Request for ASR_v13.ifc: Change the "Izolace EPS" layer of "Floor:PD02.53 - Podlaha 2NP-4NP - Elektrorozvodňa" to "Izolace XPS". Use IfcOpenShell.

First a look at what the model holds.

```python
import ifcopenshell
import ifcopenshell.util.element

model = ifcopenshell.open("ASR_v13.ifc")
print(model.schema)
for layer_set in model.by_type("IfcMaterialLayerSet"):
    if layer_set.LayerSetName == "Floor:PD02.53 - Podlaha 2NP-4NP - Elektrorozvodňa":
        for layer in layer_set.MaterialLayers:
            print(layer.id(), layer.Material and layer.Material.Name, layer.LayerThickness, sep=" | ")
        print(len(ifcopenshell.util.element.get_elements_by_material(model, layer_set)), "elements and types use it")
print(sorted(m.Name for m in model.by_type("IfcMaterial") if m.Name)[:60])
```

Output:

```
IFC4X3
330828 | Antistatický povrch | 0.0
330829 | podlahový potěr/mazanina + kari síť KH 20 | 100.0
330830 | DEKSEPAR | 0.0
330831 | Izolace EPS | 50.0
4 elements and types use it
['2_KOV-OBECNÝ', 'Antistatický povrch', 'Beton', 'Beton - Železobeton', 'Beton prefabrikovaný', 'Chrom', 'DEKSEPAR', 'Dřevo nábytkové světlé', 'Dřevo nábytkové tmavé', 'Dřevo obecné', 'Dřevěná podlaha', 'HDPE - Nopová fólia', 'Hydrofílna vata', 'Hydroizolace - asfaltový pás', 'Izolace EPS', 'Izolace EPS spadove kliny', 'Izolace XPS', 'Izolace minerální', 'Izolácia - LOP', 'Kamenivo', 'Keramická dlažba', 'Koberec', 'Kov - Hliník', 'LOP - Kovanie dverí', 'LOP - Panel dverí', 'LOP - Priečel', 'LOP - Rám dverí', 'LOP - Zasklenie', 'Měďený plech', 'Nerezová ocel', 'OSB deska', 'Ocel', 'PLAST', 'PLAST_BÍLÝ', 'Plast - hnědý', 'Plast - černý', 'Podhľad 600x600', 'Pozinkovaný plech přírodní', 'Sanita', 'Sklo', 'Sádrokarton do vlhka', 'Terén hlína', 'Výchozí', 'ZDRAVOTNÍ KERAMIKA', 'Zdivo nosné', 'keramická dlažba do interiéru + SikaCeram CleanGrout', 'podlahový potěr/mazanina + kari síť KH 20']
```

```python
import ifcopenshell
import ifcopenshell.api.material

model = ifcopenshell.open("ASR_v13.ifc")

layer_set = next(s for s in model.by_type("IfcMaterialLayerSet") if s.LayerSetName == "Floor:PD02.53 - Podlaha 2NP-4NP - Elektrorozvodňa")
layer = next(l for l in layer_set.MaterialLayers if l.Material and l.Material.Name == "Izolace EPS")
material = next(m for m in model.by_type("IfcMaterial") if m.Name == "Izolace XPS")

# Point this one layer at the other material; renaming the old one would change it everywhere.
ifcopenshell.api.material.edit_layer(model, layer=layer, attributes={"Name": material.Name}, material=material)

print([l.Material.Name if l.Material else None for l in layer_set.MaterialLayers])

model.write("ASR_v13_rev.ifc")
```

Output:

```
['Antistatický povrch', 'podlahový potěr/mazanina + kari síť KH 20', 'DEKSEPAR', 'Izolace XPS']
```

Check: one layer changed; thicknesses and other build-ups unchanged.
